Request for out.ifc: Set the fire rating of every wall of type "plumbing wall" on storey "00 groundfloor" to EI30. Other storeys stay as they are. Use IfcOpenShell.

First a look at what the model holds.

```python
import ifcopenshell
import ifcopenshell.util.element

model = ifcopenshell.open("out.ifc")
print(model.schema)
storey = next(s for s in model.by_type("IfcBuildingStorey") if s.Name == "00 groundfloor")
walls = [e for e in ifcopenshell.util.element.get_decomposition(storey) if e.is_a("IfcWall")]
seen = {}
for e in walls:
    element_type = ifcopenshell.util.element.get_type(e)
    key = (element_type.Name if element_type != e and element_type else None, ifcopenshell.util.element.get_pset(e, "Pset_WallCommon", "FireRating"))
    seen[key] = seen.get(key, 0) + 1
for (name, value), count in sorted(seen.items(), key=str):
    print(count, "x", name, "|", value)
```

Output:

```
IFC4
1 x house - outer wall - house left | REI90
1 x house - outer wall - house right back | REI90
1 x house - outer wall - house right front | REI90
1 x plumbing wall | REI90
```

```python
import ifcopenshell
import ifcopenshell.api.pset
import ifcopenshell.util.element

model = ifcopenshell.open("out.ifc")

storey = next(s for s in model.by_type("IfcBuildingStorey") if s.Name == "00 groundfloor")
walls = [e for e in ifcopenshell.util.element.get_decomposition(storey) if e.is_a("IfcWall")]

count = 0
for e in walls:
    element_type = ifcopenshell.util.element.get_type(e)
    if element_type in (None, e) or element_type.Name != "plumbing wall":
        continue
    # add_pset returns the element's existing set when there is one.
    pset = ifcopenshell.api.pset.add_pset(model, product=e, name="Pset_WallCommon")
    ifcopenshell.api.pset.edit_pset(model, pset=pset, properties={"FireRating": "EI30"})
    count += 1

print(count, "walls updated")

model.write("out_rev.ifc")
```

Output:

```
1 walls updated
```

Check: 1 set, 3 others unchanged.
